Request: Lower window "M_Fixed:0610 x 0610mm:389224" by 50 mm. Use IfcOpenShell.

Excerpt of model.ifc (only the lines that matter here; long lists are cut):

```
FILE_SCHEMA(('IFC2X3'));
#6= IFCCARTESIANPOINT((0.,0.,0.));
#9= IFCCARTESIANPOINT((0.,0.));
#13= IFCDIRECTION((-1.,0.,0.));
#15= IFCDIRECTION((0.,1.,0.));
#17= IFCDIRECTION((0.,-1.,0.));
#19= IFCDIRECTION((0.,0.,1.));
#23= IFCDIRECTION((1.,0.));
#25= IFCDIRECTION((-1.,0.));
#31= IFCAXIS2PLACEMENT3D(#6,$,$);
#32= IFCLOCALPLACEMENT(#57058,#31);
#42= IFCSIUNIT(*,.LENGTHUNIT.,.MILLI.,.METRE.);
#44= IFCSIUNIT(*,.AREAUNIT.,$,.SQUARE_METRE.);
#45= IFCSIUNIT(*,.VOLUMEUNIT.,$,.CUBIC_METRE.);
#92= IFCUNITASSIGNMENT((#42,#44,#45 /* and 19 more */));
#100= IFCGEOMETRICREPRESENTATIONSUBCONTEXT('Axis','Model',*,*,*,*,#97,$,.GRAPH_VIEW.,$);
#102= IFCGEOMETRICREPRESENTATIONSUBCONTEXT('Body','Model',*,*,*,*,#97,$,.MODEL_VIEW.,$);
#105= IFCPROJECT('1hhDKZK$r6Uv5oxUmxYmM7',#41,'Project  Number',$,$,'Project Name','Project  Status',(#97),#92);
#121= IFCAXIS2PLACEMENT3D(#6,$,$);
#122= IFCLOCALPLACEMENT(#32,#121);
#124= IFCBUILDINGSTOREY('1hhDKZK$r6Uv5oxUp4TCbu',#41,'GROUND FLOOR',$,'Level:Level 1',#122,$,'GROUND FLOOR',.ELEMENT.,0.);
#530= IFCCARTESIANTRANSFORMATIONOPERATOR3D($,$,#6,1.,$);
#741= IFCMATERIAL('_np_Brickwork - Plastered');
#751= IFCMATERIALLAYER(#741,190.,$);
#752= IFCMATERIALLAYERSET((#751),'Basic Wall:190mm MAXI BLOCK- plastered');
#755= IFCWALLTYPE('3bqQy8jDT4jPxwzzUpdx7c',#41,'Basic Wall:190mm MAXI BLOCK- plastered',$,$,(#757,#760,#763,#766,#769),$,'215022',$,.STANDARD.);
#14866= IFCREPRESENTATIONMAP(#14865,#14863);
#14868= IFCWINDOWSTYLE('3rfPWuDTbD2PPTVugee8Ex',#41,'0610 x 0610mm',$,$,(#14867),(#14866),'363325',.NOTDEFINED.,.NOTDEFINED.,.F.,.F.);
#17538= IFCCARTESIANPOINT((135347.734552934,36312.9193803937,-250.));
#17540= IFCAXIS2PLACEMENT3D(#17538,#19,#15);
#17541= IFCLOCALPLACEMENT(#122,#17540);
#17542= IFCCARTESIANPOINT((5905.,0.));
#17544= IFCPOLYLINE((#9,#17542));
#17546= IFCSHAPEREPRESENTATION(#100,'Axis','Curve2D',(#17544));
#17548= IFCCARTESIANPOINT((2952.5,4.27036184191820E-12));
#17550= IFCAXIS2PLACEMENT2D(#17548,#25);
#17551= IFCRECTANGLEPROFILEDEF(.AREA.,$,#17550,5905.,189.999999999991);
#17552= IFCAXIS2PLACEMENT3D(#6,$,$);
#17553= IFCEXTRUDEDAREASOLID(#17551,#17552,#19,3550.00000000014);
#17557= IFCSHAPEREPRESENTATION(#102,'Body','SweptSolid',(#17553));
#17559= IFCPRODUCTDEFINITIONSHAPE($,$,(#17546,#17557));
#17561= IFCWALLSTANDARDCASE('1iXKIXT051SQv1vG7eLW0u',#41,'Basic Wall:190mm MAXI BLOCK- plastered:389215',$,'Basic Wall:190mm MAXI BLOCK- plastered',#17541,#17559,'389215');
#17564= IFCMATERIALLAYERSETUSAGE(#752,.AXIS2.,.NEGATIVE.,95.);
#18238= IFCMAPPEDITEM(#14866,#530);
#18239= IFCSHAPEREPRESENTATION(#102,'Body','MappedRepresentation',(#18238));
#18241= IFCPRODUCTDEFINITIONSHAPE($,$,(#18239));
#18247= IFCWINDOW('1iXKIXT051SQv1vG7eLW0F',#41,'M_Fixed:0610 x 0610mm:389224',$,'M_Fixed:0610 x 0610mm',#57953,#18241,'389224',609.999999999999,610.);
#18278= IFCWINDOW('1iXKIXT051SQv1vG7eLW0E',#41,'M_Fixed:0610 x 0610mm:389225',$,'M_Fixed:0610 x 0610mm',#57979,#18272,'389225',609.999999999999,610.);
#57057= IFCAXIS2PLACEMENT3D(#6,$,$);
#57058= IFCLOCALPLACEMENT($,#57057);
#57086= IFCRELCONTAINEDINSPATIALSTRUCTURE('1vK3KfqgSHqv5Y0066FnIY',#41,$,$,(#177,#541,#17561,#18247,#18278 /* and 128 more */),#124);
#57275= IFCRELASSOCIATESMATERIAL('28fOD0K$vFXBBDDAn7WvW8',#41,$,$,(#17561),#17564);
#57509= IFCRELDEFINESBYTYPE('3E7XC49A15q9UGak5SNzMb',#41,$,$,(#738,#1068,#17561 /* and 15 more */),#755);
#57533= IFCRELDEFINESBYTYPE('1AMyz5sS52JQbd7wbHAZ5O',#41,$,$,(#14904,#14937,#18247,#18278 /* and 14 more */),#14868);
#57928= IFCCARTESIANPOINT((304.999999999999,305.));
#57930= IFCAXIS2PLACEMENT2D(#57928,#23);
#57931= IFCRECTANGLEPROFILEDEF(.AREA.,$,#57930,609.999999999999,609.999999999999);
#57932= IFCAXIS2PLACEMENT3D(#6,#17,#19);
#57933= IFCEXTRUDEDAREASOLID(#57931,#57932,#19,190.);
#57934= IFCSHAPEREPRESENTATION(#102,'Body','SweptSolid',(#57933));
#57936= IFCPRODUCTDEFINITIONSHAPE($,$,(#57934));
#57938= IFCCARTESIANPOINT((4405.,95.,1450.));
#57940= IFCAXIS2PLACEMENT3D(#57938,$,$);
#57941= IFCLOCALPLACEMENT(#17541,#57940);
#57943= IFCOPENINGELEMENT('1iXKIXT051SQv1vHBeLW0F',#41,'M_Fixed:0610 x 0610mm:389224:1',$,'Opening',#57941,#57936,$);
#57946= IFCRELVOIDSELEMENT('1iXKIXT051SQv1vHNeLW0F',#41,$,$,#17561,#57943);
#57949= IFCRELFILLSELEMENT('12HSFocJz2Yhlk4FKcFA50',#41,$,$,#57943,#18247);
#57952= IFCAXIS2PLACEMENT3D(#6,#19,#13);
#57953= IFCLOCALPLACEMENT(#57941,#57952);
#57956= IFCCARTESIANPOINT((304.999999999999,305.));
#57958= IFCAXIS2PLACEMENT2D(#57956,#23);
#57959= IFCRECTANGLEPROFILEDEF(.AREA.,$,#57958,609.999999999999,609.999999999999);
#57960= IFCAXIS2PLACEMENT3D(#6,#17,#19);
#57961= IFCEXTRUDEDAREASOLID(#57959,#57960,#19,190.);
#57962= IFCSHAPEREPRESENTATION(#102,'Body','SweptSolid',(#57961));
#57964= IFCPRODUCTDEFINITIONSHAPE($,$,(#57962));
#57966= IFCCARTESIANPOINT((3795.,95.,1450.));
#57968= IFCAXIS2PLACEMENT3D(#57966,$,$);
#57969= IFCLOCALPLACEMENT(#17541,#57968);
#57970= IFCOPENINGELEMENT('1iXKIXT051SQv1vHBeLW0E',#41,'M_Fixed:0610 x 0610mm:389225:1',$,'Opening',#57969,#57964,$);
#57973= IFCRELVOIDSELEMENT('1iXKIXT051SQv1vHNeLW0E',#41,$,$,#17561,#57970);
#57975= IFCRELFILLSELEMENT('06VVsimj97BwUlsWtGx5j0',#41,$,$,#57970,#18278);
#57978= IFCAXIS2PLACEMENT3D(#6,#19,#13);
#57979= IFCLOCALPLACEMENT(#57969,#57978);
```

```python
import numpy as np
import ifcopenshell
import ifcopenshell.api.geometry
import ifcopenshell.util.placement
import ifcopenshell.util.unit

model = ifcopenshell.open("model.ifc")
unit_scale = ifcopenshell.util.unit.calculate_unit_scale(model)

window = model.by_id(18247)
opening = window.FillsVoids[0].RelatingOpeningElement
dz = -50.0

shift = np.array([0.0, 0.0, dz])
# The window is placed relative to its opening, so it follows when the opening moves.
matrix = ifcopenshell.util.placement.get_local_placement(opening.ObjectPlacement)
matrix[:3, 3] += shift
ifcopenshell.api.geometry.edit_object_placement(
    model, product=opening, matrix=matrix, is_si=False, should_transform_children=True
)

print(f"moved by {dz * unit_scale:+.3f} m")

model.write("model_rev.ifc")
```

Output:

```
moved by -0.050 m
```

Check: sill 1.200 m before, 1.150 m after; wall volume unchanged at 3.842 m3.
